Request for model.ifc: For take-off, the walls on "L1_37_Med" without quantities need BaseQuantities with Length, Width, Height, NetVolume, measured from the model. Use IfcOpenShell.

First a look at what the model holds.

```python
import ifcopenshell
import ifcopenshell.util.element
import ifcopenshell.util.unit

model = ifcopenshell.open("model.ifc")
print(model.schema)
for unit_type in ("LENGTHUNIT", "AREAUNIT", "VOLUMEUNIT"):
    print(unit_type, ifcopenshell.util.unit.calculate_unit_scale(model, unit_type))
storey = next(s for s in model.by_type("IfcBuildingStorey") if s.Name == "L1_37_Med")
walls = [e for e in ifcopenshell.util.element.get_decomposition(storey) if e.is_a("IfcWall")]
for e in sorted(walls, key=lambda e: e.id()):
    print(e.id(), e.is_a(), e.Name, list(ifcopenshell.util.element.get_psets(e, qtos_only=True)), sep=" | ")
```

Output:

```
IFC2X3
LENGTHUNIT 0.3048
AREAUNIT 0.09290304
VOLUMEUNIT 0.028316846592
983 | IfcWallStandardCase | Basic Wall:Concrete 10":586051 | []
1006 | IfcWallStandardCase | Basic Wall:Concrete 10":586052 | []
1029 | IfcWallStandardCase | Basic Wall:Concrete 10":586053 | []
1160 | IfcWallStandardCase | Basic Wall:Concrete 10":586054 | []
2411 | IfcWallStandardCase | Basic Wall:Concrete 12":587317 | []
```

```python
import ifcopenshell
import ifcopenshell.api.pset
import ifcopenshell.geom
import ifcopenshell.util.element
import ifcopenshell.util.shape
import ifcopenshell.util.unit

model = ifcopenshell.open("model.ifc")
unit_scale = ifcopenshell.util.unit.calculate_unit_scale(model)
volume_scale = ifcopenshell.util.unit.calculate_unit_scale(model, "VOLUMEUNIT")
settings = ifcopenshell.geom.settings()

storey = next(s for s in model.by_type("IfcBuildingStorey") if s.Name == "L1_37_Med")
walls = [e for e in ifcopenshell.util.element.get_decomposition(storey) if e.is_a("IfcWall")]

for e in sorted(walls, key=lambda e: e.id()):
    if ifcopenshell.util.element.get_psets(e, qtos_only=True, should_inherit=False):
        continue
    # Geometry comes back in metres, in the element's own axes.
    shape = ifcopenshell.geom.create_shape(settings, e)
    values = {
        "Length": ifcopenshell.util.shape.get_x(shape.geometry) / unit_scale,
        "Width": ifcopenshell.util.shape.get_y(shape.geometry) / unit_scale,
        "Height": ifcopenshell.util.shape.get_z(shape.geometry) / unit_scale,
        "NetVolume": ifcopenshell.util.shape.get_volume(shape.geometry) / volume_scale,
    }
    qto = ifcopenshell.api.pset.add_qto(model, product=e, name="BaseQuantities")
    ifcopenshell.api.pset.edit_qto(model, qto=qto, properties=values)
    print(e.id(), {k: round(v, 3) for k, v in values.items()})

model.write("model_v2.ifc")
```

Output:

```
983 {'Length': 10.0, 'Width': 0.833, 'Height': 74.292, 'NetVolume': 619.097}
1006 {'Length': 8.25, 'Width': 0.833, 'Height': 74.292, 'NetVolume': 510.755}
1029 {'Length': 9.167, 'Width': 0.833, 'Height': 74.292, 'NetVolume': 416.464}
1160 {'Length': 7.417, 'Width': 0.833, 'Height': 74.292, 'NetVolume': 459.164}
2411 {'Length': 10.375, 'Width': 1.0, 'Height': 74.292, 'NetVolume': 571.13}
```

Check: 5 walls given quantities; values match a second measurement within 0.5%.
